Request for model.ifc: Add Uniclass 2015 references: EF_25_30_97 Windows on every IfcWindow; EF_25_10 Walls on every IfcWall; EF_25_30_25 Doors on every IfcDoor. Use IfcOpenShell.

First a look at what the model holds.

```python
import ifcopenshell

model = ifcopenshell.open("model.ifc")
print(model.schema)
print("classifications:", [c.Name for c in model.by_type("IfcClassification")])
for ifc_class in ("IfcDoor", "IfcRoof", "IfcStair", "IfcWall", "IfcWindow"):
    print(ifc_class, len(model.by_type(ifc_class)))
```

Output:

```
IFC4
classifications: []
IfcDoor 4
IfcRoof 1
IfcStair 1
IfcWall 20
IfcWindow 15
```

```python
import ifcopenshell
import ifcopenshell.api.classification

model = ifcopenshell.open("model.ifc")

system = ifcopenshell.api.classification.add_classification(model, classification="Uniclass 2015")

codes = {
    "IfcWindow": ("EF_25_30_97", "Windows"),
    "IfcWall": ("EF_25_10", "Walls"),
    "IfcDoor": ("EF_25_30_25", "Doors"),
}
for ifc_class, (code, name) in codes.items():
    products = model.by_type(ifc_class)
    ifcopenshell.api.classification.add_reference(
        model, products=products, classification=system, identification=code, name=name
    )
    print(code, len(products))

model.write("model-out.ifc")
```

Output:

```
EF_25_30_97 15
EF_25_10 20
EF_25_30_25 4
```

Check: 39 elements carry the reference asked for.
